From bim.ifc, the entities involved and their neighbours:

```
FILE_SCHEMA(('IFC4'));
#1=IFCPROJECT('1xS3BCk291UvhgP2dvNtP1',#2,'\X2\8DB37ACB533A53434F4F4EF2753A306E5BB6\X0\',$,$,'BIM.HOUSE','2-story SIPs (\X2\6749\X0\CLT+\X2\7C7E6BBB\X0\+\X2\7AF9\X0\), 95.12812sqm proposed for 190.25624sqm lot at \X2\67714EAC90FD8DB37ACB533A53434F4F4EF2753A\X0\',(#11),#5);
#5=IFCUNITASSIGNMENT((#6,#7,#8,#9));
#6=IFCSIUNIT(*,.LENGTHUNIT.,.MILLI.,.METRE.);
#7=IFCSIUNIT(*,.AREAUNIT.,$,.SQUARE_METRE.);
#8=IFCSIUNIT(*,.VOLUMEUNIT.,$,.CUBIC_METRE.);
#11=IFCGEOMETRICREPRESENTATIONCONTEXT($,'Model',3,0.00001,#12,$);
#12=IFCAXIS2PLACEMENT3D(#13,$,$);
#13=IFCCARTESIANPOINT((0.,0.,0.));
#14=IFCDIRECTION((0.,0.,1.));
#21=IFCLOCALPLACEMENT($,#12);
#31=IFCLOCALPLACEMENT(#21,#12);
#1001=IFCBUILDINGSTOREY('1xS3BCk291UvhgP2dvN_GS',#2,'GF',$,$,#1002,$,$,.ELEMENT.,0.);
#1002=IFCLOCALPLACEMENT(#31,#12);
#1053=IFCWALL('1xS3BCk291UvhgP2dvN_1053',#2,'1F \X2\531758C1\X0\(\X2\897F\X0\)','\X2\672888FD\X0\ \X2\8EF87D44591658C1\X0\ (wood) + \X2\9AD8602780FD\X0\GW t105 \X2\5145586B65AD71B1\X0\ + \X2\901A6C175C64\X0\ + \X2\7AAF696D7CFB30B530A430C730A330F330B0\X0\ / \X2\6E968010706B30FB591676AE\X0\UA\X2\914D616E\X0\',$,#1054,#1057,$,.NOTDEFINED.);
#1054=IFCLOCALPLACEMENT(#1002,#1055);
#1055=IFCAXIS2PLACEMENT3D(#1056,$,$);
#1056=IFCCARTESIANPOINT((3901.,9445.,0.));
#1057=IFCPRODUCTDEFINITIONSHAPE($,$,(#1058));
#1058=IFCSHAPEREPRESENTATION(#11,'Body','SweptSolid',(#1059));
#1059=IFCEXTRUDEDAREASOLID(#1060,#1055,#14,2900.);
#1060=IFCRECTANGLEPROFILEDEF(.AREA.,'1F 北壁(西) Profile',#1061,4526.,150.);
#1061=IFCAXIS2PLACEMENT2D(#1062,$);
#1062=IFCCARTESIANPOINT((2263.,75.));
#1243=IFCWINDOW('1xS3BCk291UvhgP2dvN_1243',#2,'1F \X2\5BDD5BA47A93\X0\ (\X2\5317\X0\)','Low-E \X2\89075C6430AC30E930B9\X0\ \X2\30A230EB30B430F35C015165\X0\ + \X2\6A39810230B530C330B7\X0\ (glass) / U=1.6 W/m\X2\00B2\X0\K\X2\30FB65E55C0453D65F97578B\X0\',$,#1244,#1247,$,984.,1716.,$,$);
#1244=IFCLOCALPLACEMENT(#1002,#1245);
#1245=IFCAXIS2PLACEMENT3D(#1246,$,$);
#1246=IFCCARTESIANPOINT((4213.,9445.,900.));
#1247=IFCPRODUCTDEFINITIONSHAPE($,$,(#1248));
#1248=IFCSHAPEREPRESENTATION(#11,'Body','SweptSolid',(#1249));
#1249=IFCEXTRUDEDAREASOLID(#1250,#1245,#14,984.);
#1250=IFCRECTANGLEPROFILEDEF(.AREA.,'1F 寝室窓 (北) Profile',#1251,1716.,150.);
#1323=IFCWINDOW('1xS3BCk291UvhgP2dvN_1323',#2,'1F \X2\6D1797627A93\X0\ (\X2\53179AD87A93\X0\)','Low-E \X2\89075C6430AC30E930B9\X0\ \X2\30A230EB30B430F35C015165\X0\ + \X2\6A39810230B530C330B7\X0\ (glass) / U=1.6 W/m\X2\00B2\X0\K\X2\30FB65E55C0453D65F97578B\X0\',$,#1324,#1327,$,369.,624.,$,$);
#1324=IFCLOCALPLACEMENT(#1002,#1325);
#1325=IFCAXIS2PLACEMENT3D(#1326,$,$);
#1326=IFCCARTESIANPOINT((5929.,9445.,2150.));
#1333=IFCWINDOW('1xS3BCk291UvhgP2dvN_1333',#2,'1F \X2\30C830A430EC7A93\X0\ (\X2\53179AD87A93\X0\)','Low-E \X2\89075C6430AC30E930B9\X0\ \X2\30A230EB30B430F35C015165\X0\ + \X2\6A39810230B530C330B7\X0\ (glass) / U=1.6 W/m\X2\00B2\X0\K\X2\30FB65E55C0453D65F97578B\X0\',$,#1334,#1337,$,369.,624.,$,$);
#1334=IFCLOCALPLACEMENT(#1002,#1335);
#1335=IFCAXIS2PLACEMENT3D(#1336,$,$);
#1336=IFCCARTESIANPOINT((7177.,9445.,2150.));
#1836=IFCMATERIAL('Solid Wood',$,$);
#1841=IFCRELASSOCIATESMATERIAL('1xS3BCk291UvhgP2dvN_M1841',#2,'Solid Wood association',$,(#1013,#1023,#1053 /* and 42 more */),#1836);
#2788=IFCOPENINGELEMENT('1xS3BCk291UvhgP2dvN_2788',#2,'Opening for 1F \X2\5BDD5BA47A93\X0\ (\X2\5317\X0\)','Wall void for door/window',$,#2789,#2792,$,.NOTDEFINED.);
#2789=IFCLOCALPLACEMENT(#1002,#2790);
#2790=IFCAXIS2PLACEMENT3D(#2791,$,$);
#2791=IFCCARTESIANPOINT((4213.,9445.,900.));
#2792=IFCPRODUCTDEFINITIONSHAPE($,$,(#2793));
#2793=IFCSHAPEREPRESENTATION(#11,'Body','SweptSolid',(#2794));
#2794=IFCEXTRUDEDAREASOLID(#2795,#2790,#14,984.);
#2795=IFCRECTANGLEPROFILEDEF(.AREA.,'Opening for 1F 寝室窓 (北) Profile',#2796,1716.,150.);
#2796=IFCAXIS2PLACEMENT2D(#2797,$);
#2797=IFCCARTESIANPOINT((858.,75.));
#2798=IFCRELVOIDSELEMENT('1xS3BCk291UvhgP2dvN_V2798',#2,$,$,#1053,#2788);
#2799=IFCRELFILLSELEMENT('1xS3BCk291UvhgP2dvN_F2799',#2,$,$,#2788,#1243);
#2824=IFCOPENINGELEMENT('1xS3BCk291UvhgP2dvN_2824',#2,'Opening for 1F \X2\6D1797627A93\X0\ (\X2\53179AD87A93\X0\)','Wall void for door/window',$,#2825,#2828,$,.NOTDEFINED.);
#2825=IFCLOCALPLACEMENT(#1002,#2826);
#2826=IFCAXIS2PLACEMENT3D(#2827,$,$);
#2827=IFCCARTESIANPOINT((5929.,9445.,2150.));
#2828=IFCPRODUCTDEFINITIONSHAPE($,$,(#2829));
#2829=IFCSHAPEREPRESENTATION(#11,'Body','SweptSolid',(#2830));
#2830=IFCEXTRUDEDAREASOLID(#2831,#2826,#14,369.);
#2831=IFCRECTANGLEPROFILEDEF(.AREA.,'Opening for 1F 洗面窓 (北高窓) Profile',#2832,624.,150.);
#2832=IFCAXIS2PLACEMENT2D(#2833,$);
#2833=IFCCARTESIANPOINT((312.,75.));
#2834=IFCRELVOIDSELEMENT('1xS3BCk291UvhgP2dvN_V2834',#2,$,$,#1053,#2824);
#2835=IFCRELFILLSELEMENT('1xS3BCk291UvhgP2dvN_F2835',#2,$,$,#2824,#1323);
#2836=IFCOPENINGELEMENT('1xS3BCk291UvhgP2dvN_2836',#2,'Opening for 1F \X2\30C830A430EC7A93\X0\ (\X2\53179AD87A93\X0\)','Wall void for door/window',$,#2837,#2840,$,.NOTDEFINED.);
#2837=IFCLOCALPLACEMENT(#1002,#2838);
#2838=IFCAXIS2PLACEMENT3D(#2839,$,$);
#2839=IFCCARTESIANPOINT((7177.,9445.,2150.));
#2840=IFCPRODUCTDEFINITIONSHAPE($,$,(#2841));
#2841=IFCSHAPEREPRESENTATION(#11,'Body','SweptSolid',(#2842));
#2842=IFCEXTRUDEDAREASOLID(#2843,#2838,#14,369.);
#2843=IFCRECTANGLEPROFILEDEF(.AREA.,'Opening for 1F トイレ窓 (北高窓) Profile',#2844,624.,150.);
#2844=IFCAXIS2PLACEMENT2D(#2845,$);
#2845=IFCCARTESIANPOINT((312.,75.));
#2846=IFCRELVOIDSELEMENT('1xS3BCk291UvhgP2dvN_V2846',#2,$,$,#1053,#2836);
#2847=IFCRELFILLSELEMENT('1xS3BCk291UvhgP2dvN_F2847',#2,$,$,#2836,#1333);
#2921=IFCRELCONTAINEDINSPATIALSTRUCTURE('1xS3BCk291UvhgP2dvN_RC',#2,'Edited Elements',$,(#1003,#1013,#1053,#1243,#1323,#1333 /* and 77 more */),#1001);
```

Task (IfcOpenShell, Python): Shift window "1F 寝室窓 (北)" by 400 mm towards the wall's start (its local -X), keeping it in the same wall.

```python
import ifcopenshell
import ifcopenshell.api.geometry
import ifcopenshell.util.placement
import ifcopenshell.util.unit

model = ifcopenshell.open("bim.ifc")
unit_scale = ifcopenshell.util.unit.calculate_unit_scale(model)

window = model.by_guid("1xS3BCk291UvhgP2dvN_1243")
opening = window.FillsVoids[0].RelatingOpeningElement
wall = opening.VoidsElements[0].RelatingBuildingElement

wall_matrix = ifcopenshell.util.placement.get_local_placement(wall.ObjectPlacement)
shift = wall_matrix[:3, 0] * -0.4 / unit_scale
before = ifcopenshell.util.placement.get_local_placement(window.ObjectPlacement)[:3, 3].copy()

# The window is not placed relative to its opening, so move both.
for product in (opening, window):
    matrix = ifcopenshell.util.placement.get_local_placement(product.ObjectPlacement)
    matrix[:3, 3] += shift
    ifcopenshell.api.geometry.edit_object_placement(model, product=product, matrix=matrix, is_si=False)

after = ifcopenshell.util.placement.get_local_placement(window.ObjectPlacement)[:3, 3]
print("window moved by", (after - before).round(3) + 0.0)

model.write("bim_updated.ifc")
```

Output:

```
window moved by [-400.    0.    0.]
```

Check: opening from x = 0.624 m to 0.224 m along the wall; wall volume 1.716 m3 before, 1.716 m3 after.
